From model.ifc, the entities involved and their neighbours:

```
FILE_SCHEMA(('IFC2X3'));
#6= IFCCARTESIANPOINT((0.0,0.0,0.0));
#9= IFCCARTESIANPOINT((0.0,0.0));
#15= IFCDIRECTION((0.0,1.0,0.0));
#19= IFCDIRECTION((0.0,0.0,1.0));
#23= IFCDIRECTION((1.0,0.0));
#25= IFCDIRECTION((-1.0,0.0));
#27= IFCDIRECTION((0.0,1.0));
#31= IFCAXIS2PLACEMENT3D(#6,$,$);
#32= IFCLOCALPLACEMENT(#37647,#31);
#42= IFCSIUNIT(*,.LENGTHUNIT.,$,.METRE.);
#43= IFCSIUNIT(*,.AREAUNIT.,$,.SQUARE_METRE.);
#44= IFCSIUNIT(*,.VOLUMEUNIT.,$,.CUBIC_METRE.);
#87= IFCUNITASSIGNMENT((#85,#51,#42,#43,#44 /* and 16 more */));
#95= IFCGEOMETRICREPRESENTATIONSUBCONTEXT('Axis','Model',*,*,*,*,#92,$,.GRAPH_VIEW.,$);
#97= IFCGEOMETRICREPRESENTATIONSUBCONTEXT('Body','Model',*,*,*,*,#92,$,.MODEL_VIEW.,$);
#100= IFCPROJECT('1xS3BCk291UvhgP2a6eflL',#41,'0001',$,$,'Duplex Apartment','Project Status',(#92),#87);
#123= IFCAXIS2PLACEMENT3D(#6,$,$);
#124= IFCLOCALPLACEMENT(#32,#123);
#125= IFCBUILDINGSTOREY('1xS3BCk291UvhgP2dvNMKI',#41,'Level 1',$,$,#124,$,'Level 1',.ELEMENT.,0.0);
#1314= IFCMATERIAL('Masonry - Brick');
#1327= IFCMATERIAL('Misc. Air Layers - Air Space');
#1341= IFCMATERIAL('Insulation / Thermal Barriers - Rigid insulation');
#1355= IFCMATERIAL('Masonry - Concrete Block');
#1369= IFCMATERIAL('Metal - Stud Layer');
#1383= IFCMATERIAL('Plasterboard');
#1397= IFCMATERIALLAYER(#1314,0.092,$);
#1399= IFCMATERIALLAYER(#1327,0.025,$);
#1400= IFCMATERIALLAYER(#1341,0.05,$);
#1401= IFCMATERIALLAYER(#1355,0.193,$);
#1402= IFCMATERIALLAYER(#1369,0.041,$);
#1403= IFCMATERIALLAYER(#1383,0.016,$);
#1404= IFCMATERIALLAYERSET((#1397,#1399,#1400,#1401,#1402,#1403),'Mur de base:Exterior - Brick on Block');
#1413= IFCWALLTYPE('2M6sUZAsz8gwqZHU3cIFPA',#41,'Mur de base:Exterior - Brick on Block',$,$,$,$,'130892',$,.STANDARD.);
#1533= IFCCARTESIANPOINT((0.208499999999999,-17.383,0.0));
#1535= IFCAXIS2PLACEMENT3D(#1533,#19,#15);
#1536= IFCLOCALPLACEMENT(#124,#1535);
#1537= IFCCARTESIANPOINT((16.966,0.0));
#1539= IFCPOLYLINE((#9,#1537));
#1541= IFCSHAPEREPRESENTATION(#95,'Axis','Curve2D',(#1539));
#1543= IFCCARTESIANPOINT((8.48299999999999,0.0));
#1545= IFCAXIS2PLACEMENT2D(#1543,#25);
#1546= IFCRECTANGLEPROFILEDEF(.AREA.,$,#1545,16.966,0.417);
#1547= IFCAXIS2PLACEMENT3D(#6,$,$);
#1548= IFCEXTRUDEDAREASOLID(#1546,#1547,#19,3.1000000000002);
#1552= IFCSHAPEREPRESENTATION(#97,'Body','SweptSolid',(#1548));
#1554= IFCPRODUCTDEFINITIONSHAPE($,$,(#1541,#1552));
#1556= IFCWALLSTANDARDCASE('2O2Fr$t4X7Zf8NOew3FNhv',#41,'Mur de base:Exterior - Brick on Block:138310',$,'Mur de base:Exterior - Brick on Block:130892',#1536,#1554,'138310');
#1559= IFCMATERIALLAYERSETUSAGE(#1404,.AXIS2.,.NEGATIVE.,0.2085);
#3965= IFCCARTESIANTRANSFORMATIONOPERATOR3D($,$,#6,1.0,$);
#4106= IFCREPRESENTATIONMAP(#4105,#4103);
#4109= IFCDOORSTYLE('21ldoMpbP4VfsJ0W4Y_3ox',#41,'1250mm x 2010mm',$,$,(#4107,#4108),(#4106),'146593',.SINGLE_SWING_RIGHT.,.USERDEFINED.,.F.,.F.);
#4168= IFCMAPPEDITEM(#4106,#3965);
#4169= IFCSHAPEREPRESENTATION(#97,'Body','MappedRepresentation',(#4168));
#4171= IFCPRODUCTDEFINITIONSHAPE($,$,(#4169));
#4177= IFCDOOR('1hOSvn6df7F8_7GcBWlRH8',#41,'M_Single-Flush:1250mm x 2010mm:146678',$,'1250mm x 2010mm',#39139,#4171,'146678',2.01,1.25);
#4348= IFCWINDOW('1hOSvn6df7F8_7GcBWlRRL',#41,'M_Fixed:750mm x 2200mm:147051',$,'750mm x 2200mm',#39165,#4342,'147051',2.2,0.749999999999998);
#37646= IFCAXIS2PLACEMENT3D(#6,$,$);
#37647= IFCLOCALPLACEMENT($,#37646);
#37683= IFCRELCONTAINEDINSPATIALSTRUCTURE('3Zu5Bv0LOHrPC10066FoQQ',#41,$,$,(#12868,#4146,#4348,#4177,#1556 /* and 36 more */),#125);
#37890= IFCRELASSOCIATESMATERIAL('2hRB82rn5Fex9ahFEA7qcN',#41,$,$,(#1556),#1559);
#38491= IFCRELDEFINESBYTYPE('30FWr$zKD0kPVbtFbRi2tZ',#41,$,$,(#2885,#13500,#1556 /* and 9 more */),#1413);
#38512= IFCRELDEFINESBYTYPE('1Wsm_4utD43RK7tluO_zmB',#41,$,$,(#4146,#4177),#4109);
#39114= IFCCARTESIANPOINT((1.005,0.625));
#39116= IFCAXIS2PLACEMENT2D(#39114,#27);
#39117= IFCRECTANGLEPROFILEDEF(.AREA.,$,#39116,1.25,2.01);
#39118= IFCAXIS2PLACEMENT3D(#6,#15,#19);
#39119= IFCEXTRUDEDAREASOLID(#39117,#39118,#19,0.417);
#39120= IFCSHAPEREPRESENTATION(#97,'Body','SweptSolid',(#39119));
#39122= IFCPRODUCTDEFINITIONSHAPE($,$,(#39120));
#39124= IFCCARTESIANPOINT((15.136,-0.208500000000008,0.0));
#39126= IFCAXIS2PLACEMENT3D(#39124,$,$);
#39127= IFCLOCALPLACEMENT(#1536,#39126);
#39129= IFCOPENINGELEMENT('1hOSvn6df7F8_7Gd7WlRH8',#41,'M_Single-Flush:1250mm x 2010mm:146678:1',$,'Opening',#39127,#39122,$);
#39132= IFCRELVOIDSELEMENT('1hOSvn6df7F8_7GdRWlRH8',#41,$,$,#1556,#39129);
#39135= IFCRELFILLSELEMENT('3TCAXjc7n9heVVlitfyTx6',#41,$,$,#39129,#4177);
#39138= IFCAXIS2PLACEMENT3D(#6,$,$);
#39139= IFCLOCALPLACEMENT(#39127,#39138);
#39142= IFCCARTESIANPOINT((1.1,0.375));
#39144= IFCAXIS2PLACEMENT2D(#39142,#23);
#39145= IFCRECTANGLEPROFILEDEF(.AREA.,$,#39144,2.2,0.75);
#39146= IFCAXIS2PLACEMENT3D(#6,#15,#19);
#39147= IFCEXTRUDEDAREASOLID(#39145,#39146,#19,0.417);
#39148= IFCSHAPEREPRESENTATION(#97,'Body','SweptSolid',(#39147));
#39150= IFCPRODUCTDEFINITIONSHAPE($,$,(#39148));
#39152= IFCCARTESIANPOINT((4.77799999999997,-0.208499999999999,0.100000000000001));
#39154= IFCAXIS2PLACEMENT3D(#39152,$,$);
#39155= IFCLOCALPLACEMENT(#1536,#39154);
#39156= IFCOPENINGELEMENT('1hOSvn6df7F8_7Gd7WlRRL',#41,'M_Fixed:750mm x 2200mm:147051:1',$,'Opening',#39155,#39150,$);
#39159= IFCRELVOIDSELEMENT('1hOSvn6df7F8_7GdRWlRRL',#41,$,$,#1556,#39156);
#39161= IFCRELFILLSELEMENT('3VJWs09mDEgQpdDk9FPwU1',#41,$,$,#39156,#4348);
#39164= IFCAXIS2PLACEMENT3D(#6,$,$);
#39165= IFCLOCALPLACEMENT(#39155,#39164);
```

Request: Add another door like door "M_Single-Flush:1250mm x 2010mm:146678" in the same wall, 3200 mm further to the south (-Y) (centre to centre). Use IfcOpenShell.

```python
import ifcopenshell
import ifcopenshell.api.feature
import ifcopenshell.api.geometry
import ifcopenshell.api.root
import ifcopenshell.geom
import ifcopenshell.util.element
import ifcopenshell.util.placement
import ifcopenshell.util.shape
import ifcopenshell.util.unit

model = ifcopenshell.open("model.ifc")
unit_scale = ifcopenshell.util.unit.calculate_unit_scale(model)
settings = ifcopenshell.geom.settings()


def volume(element):
    """Net volume in cubic metres, openings subtracted."""
    shape = ifcopenshell.geom.create_shape(settings, element)
    return ifcopenshell.util.shape.get_volume(shape.geometry)


def reuse_history(source, copy):
    """copy_class also copies each property set's owner history, people and application; keep the originals."""
    for rel in copy.IsDefinedBy:
        if rel.is_a("IfcRelDefinesByProperties") and (history := rel.RelatingPropertyDefinition.OwnerHistory):
            rel.RelatingPropertyDefinition.OwnerHistory = source.OwnerHistory
            ifcopenshell.util.element.remove_deep2(model, history)


door = model.by_id(4177)
opening = door.FillsVoids[0].RelatingOpeningElement
wall = opening.VoidsElements[0].RelatingBuildingElement
before = volume(wall)
shift = ifcopenshell.util.placement.get_local_placement(wall.ObjectPlacement)[:3, 0] * -3.2 / unit_scale

# copy_class copies the void relationship, type, container and properties, but no geometry.
new_opening = ifcopenshell.api.root.copy_class(model, product=opening)
new_opening.Representation = ifcopenshell.util.element.copy_deep(
    model, opening.Representation, exclude=["IfcGeometricRepresentationContext", "IfcRepresentationMap"]
)
new_opening.Name = "M_Single-Flush:1250mm x 2010mm"
new_door = ifcopenshell.api.root.copy_class(model, product=door)
new_door.Representation = ifcopenshell.util.element.copy_deep(
    model, door.Representation, exclude=["IfcGeometricRepresentationContext", "IfcRepresentationMap"]
)
new_door.Name = "M_Single-Flush:1250mm x 2010mm"
new_door.Tag = None
reuse_history(door, new_door)
fills = ifcopenshell.api.feature.add_filling(model, opening=new_opening, element=new_door)
fills.OwnerHistory = new_door.OwnerHistory  # required in IFC2X3

for old, new in ((opening, new_opening), (door, new_door)):
    matrix = ifcopenshell.util.placement.get_local_placement(old.ObjectPlacement)
    matrix[:3, 3] += shift
    ifcopenshell.api.geometry.edit_object_placement(model, product=new, matrix=matrix, is_si=False)

after = volume(wall)

print(f"wall volume {before:.3f} -> {after:.3f} m3")

model.write("model_rev.ifc")
```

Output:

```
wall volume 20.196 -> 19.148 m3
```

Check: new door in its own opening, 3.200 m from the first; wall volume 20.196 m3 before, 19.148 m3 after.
